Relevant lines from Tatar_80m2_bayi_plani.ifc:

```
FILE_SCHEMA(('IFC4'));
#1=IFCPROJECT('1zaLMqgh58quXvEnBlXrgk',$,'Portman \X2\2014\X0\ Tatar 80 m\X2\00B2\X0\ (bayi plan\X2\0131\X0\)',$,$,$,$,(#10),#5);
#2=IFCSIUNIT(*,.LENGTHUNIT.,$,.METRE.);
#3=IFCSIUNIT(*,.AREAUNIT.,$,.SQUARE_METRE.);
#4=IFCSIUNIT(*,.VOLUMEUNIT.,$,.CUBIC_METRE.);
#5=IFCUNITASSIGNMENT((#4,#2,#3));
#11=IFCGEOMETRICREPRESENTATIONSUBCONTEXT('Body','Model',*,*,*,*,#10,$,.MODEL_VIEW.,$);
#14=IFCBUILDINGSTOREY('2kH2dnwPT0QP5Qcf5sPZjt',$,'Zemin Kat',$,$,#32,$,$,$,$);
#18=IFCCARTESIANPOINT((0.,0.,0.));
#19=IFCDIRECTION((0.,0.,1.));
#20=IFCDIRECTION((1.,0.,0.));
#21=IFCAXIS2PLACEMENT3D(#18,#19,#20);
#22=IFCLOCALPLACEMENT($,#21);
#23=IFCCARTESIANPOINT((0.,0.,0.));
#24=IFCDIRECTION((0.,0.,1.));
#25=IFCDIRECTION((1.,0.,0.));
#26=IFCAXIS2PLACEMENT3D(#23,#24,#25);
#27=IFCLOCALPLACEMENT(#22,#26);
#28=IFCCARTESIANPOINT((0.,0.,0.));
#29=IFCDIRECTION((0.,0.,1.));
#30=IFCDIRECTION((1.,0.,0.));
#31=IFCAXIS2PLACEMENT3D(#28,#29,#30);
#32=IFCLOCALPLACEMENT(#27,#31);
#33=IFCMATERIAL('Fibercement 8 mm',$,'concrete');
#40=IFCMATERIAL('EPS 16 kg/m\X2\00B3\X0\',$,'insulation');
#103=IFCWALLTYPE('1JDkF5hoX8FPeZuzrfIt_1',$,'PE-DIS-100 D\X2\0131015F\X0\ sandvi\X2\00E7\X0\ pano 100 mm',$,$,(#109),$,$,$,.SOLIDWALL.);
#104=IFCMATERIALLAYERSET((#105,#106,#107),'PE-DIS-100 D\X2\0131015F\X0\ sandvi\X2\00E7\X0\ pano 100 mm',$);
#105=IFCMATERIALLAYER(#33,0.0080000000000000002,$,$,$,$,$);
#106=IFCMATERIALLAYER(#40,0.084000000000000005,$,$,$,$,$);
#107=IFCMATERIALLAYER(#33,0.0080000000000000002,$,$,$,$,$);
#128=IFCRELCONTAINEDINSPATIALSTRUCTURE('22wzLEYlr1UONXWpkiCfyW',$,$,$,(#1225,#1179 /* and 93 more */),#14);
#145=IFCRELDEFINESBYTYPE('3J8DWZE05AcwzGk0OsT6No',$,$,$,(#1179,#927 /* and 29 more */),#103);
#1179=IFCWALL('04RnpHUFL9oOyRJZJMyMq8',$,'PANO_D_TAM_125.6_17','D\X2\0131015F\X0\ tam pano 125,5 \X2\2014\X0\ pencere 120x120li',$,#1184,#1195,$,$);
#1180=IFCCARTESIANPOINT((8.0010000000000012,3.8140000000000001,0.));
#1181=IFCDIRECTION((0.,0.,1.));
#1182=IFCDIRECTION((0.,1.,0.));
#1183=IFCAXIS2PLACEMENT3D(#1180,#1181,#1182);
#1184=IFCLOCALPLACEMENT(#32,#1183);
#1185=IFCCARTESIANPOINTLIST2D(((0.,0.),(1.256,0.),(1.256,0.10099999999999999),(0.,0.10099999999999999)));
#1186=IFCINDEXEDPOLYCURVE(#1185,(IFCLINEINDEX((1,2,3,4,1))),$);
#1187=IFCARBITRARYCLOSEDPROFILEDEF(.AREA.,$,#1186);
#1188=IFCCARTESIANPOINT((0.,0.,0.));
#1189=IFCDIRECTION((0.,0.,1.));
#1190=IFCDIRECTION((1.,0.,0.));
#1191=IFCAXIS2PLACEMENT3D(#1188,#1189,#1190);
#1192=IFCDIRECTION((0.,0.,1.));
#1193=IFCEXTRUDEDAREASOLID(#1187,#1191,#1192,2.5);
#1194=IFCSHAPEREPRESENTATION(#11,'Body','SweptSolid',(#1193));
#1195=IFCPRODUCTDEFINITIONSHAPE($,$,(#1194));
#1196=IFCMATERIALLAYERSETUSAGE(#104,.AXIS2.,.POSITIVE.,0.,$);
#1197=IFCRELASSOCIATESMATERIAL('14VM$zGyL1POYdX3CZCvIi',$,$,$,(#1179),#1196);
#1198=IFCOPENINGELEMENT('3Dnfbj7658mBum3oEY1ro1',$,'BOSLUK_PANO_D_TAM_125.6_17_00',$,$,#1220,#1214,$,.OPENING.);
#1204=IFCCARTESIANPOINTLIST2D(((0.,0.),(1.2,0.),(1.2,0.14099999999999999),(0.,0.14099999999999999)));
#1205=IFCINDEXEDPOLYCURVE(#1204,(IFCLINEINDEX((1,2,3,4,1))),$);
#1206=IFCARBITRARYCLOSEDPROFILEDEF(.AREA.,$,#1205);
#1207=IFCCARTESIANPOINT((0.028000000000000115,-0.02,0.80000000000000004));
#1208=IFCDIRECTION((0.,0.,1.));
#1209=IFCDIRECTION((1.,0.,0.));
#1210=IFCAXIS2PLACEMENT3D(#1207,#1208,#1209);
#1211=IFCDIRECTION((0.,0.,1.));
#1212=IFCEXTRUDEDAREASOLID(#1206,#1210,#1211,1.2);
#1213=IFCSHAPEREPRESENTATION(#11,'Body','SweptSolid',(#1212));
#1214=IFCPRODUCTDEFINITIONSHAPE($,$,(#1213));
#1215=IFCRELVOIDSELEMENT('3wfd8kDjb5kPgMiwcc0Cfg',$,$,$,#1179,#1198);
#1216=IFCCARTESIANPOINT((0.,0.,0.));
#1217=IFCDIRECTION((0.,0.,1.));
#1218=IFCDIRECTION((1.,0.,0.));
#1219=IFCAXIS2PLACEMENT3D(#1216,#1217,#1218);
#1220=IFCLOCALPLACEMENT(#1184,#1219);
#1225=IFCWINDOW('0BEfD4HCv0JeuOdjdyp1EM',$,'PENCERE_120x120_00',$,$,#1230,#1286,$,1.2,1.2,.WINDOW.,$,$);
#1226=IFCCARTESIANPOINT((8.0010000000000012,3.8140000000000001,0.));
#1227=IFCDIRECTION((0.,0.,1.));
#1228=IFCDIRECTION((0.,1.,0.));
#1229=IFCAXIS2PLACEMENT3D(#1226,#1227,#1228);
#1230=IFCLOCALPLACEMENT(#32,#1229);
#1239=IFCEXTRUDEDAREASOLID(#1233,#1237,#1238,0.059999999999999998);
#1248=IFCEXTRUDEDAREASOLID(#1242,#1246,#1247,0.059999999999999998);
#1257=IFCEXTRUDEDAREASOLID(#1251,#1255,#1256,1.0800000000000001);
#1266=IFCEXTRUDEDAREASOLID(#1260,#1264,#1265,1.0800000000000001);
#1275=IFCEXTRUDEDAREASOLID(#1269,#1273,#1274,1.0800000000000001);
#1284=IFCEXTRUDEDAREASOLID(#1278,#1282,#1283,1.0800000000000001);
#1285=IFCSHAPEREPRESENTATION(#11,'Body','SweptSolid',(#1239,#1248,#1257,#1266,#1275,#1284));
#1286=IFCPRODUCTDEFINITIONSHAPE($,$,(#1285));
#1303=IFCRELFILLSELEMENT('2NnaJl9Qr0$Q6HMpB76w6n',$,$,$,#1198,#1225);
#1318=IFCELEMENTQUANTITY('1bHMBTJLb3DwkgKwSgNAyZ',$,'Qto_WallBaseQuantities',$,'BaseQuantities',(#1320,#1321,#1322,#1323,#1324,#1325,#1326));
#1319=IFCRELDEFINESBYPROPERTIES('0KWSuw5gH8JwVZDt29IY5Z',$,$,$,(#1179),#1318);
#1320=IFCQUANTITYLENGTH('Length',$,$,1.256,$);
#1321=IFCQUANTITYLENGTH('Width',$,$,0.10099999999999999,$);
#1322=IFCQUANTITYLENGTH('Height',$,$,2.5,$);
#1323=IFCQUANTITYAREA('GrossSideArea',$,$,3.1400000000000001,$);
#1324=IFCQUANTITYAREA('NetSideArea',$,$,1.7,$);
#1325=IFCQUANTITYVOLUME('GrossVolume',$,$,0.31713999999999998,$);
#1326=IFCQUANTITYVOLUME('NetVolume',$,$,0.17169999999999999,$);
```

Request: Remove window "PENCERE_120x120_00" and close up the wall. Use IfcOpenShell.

```python
import ifcopenshell
import ifcopenshell.api.feature
import ifcopenshell.api.pset
import ifcopenshell.api.root
import ifcopenshell.geom
import ifcopenshell.util.element
import ifcopenshell.util.shape
import ifcopenshell.util.unit

model = ifcopenshell.open("Tatar_80m2_bayi_plani.ifc")
area_scale = ifcopenshell.util.unit.calculate_unit_scale(model, "AREAUNIT")
volume_scale = ifcopenshell.util.unit.calculate_unit_scale(model, "VOLUMEUNIT")
settings = ifcopenshell.geom.settings()


def volume(element):
    """Net volume in cubic metres, openings subtracted."""
    shape = ifcopenshell.geom.create_shape(settings, element)
    return ifcopenshell.util.shape.get_volume(shape.geometry)


window = model.by_id(1225)
opening = window.FillsVoids[0].RelatingOpeningElement
wall = opening.VoidsElements[0].RelatingBuildingElement
before = volume(wall)

ifcopenshell.api.root.remove_product(model, product=window)
ifcopenshell.api.feature.remove_feature(model, feature=opening)

after = volume(wall)
thickness = 0.101  # wall thickness in metres

# Update the wall's stored quantities.
qto = model.by_id(ifcopenshell.util.element.get_pset(wall, "Qto_WallBaseQuantities", should_inherit=False)["id"])
ifcopenshell.api.pset.edit_qto(model, qto=qto, properties={
    "NetSideArea": after / thickness / area_scale,
    "NetVolume": after / volume_scale,
})

print(f"wall volume {before:.3f} -> {after:.3f} m3")

model.write("Tatar_80m2_bayi_plani_rev.ifc")
```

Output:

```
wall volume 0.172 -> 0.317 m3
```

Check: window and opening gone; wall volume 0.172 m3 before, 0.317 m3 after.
